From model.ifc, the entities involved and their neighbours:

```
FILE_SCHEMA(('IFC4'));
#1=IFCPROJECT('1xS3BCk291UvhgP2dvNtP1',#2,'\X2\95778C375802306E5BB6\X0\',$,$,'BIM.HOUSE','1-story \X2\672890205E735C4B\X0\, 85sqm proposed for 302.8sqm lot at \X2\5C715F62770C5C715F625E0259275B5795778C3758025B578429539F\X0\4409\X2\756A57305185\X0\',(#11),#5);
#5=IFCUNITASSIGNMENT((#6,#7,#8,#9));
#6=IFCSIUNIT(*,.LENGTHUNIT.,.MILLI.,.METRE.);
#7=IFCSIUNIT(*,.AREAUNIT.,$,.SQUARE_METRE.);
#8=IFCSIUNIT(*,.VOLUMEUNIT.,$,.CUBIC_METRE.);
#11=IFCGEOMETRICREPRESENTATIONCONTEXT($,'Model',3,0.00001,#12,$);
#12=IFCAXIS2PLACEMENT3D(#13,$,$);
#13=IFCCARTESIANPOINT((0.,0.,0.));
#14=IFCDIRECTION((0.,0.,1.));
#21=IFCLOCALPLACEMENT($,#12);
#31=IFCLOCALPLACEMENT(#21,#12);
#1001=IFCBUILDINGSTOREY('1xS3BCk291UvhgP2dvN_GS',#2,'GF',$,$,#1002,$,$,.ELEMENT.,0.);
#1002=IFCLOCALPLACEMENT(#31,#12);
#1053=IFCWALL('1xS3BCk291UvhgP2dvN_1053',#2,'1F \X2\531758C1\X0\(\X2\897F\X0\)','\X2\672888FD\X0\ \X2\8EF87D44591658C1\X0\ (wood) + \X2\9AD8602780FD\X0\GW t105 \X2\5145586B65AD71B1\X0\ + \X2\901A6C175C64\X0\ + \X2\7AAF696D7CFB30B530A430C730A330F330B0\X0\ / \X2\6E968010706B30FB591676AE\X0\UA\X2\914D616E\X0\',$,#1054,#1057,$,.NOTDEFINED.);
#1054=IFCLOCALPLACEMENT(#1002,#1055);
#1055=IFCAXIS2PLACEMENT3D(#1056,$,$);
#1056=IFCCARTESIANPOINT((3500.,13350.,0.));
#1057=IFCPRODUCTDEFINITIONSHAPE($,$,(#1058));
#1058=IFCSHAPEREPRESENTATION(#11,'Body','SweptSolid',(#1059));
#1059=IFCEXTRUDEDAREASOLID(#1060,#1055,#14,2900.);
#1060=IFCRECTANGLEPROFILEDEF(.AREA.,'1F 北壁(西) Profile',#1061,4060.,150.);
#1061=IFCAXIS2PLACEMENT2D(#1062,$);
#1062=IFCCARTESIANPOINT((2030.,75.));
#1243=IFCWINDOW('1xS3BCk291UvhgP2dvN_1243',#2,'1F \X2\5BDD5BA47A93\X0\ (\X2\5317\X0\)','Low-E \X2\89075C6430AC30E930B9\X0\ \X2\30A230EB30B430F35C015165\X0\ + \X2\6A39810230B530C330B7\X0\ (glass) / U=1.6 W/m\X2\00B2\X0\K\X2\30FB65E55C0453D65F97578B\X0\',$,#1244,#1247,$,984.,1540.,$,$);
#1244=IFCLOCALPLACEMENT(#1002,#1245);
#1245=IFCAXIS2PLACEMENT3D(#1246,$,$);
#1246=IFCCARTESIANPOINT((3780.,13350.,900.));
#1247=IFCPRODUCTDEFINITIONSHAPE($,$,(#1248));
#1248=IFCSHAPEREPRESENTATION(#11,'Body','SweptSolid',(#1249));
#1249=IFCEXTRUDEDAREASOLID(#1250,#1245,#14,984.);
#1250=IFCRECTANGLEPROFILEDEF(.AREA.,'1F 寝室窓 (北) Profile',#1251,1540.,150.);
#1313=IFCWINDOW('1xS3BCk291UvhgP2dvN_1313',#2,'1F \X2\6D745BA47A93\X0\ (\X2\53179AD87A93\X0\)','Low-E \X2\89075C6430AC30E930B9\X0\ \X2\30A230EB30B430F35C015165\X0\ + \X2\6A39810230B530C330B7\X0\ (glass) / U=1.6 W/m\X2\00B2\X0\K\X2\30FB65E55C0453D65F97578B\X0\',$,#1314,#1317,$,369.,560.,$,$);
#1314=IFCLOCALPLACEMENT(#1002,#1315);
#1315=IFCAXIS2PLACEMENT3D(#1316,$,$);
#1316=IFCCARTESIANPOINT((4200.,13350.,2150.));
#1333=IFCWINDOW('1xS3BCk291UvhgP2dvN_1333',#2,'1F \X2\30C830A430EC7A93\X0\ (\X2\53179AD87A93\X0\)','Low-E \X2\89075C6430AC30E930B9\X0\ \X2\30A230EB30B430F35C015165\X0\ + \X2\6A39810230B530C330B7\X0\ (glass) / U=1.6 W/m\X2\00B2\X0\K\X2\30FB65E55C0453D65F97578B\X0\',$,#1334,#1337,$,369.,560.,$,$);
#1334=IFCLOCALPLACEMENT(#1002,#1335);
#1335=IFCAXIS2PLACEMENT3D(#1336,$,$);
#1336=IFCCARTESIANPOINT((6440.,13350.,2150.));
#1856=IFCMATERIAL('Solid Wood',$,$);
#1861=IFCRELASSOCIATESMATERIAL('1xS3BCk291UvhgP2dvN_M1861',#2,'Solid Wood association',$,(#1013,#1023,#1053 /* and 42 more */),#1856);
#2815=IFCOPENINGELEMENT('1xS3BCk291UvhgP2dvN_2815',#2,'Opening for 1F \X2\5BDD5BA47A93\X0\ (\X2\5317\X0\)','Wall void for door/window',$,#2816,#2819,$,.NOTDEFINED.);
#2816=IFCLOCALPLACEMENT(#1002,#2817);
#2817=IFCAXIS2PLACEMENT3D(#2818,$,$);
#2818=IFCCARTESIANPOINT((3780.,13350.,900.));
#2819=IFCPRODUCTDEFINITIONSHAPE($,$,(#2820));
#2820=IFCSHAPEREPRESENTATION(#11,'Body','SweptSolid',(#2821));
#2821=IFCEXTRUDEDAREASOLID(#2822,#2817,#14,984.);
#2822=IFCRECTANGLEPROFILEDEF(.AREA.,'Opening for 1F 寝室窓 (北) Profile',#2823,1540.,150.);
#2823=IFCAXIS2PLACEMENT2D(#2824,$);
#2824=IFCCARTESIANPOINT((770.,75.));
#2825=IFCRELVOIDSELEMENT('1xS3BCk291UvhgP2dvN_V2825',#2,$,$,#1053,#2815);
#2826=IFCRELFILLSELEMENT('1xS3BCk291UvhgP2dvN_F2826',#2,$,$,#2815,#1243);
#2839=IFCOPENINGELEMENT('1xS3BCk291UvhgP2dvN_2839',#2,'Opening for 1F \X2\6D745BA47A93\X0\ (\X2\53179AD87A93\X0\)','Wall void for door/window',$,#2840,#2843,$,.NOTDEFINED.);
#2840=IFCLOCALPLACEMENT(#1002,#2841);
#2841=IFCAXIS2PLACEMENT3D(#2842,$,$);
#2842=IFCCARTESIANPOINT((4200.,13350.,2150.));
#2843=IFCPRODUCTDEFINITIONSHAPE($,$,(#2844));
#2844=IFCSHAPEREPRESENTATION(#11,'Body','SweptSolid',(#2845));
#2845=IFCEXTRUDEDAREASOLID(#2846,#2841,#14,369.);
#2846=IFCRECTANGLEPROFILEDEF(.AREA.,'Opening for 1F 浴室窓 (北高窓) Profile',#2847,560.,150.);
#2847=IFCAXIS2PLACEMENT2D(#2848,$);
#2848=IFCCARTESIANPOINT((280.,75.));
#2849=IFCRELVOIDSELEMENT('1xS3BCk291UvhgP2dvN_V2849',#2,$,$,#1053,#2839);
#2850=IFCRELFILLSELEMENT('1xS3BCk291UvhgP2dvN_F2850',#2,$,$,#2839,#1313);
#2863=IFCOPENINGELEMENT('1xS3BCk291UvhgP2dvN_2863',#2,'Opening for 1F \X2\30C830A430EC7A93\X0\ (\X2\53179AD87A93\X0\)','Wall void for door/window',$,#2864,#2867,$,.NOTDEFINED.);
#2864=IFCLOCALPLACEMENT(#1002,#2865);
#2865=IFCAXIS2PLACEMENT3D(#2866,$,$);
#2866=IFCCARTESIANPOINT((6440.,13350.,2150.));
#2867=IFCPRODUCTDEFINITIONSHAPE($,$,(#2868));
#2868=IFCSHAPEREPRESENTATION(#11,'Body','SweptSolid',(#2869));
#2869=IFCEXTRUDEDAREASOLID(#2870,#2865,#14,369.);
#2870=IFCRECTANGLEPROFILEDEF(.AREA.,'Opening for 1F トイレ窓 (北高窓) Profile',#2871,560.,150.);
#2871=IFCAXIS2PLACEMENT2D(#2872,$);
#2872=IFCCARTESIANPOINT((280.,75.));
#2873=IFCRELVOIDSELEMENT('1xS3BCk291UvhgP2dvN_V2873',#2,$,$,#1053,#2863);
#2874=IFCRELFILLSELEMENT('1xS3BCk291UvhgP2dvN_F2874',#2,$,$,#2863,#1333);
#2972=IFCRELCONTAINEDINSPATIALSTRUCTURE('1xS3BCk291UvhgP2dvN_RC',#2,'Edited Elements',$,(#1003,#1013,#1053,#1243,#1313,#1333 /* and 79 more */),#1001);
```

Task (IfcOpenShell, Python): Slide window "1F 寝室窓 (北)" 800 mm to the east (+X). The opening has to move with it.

```python
import ifcopenshell
import ifcopenshell.api.geometry
import ifcopenshell.util.placement
import ifcopenshell.util.unit

model = ifcopenshell.open("model.ifc")
unit_scale = ifcopenshell.util.unit.calculate_unit_scale(model)

window = model.by_guid("1xS3BCk291UvhgP2dvN_1243")
opening = window.FillsVoids[0].RelatingOpeningElement
wall = opening.VoidsElements[0].RelatingBuildingElement

wall_matrix = ifcopenshell.util.placement.get_local_placement(wall.ObjectPlacement)
shift = wall_matrix[:3, 0] * 0.8 / unit_scale
before = ifcopenshell.util.placement.get_local_placement(window.ObjectPlacement)[:3, 3].copy()

# The window is not placed relative to its opening, so move both.
for product in (opening, window):
    matrix = ifcopenshell.util.placement.get_local_placement(product.ObjectPlacement)
    matrix[:3, 3] += shift
    ifcopenshell.api.geometry.edit_object_placement(model, product=product, matrix=matrix, is_si=False)

after = ifcopenshell.util.placement.get_local_placement(window.ObjectPlacement)[:3, 3]
print("window moved by", (after - before).round(3) + 0.0)

model.write("model_rev.ifc")
```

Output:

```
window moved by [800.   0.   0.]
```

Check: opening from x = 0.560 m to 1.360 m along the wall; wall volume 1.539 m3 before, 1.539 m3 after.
